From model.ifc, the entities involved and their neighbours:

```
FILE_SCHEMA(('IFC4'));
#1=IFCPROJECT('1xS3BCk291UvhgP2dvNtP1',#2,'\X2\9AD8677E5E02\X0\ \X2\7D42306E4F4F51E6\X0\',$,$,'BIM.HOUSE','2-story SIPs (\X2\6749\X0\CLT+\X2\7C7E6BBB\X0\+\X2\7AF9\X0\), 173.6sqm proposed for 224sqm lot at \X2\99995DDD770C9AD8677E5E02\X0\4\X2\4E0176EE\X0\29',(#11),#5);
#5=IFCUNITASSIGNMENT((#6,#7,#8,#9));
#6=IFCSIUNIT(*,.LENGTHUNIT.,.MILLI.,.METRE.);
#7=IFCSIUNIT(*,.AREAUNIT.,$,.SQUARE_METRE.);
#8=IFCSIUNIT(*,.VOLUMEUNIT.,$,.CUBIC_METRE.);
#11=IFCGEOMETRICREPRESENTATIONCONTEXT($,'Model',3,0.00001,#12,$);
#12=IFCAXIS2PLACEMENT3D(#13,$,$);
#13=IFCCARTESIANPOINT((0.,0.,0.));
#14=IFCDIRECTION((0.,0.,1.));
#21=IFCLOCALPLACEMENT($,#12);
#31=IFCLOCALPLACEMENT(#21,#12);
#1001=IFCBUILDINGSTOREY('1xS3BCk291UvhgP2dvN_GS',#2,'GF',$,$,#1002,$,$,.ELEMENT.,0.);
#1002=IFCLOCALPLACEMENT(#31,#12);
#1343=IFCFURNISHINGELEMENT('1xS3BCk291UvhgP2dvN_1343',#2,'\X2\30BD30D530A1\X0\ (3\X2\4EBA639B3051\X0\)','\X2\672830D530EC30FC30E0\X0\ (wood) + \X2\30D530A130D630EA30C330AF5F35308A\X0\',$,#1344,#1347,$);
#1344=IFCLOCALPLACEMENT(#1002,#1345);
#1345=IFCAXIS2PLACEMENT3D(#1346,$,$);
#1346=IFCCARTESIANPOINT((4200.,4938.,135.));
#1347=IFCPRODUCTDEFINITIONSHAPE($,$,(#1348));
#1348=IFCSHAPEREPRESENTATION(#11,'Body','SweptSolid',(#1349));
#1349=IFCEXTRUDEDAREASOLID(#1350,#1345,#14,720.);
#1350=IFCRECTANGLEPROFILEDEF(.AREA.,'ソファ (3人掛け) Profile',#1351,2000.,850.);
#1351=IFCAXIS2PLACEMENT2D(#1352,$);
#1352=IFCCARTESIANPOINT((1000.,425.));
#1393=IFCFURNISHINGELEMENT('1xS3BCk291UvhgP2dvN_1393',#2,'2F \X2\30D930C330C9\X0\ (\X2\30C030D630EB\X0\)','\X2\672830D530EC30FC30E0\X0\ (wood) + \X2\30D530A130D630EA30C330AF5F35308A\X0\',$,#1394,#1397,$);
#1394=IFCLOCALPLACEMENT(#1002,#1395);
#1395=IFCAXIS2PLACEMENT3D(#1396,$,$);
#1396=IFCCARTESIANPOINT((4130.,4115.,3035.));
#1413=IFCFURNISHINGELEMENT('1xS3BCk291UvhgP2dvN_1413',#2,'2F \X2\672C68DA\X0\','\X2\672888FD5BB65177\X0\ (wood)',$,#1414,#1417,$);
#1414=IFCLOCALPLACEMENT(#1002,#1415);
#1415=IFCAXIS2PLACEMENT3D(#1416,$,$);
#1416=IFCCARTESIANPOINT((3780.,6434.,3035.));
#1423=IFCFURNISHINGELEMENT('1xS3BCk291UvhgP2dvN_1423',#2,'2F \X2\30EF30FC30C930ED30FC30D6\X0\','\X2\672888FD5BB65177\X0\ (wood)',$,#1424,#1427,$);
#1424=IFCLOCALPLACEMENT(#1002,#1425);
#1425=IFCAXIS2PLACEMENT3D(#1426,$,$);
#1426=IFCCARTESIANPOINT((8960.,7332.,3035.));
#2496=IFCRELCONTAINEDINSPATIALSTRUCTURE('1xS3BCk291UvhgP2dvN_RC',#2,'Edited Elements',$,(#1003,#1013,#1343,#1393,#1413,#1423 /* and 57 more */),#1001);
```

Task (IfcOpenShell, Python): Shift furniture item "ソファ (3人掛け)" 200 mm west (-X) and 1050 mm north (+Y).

```python
import ifcopenshell
import ifcopenshell.api.geometry
import ifcopenshell.util.placement
import ifcopenshell.util.unit

model = ifcopenshell.open("model.ifc")
unit_scale = ifcopenshell.util.unit.calculate_unit_scale(model)

item = model.by_id(1343)
matrix = ifcopenshell.util.placement.get_local_placement(item.ObjectPlacement)
matrix[0, 3] -= 0.2 / unit_scale
matrix[1, 3] += 1.05 / unit_scale
ifcopenshell.api.geometry.edit_object_placement(model, product=item, matrix=matrix, is_si=False)

print(ifcopenshell.util.placement.get_local_placement(item.ObjectPlacement).round(3) + 0.0)

model.write("model_v2.ifc")
```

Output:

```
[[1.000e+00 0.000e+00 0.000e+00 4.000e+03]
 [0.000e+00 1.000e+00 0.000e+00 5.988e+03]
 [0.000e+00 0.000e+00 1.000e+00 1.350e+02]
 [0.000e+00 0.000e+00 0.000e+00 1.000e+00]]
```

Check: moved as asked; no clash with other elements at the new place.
